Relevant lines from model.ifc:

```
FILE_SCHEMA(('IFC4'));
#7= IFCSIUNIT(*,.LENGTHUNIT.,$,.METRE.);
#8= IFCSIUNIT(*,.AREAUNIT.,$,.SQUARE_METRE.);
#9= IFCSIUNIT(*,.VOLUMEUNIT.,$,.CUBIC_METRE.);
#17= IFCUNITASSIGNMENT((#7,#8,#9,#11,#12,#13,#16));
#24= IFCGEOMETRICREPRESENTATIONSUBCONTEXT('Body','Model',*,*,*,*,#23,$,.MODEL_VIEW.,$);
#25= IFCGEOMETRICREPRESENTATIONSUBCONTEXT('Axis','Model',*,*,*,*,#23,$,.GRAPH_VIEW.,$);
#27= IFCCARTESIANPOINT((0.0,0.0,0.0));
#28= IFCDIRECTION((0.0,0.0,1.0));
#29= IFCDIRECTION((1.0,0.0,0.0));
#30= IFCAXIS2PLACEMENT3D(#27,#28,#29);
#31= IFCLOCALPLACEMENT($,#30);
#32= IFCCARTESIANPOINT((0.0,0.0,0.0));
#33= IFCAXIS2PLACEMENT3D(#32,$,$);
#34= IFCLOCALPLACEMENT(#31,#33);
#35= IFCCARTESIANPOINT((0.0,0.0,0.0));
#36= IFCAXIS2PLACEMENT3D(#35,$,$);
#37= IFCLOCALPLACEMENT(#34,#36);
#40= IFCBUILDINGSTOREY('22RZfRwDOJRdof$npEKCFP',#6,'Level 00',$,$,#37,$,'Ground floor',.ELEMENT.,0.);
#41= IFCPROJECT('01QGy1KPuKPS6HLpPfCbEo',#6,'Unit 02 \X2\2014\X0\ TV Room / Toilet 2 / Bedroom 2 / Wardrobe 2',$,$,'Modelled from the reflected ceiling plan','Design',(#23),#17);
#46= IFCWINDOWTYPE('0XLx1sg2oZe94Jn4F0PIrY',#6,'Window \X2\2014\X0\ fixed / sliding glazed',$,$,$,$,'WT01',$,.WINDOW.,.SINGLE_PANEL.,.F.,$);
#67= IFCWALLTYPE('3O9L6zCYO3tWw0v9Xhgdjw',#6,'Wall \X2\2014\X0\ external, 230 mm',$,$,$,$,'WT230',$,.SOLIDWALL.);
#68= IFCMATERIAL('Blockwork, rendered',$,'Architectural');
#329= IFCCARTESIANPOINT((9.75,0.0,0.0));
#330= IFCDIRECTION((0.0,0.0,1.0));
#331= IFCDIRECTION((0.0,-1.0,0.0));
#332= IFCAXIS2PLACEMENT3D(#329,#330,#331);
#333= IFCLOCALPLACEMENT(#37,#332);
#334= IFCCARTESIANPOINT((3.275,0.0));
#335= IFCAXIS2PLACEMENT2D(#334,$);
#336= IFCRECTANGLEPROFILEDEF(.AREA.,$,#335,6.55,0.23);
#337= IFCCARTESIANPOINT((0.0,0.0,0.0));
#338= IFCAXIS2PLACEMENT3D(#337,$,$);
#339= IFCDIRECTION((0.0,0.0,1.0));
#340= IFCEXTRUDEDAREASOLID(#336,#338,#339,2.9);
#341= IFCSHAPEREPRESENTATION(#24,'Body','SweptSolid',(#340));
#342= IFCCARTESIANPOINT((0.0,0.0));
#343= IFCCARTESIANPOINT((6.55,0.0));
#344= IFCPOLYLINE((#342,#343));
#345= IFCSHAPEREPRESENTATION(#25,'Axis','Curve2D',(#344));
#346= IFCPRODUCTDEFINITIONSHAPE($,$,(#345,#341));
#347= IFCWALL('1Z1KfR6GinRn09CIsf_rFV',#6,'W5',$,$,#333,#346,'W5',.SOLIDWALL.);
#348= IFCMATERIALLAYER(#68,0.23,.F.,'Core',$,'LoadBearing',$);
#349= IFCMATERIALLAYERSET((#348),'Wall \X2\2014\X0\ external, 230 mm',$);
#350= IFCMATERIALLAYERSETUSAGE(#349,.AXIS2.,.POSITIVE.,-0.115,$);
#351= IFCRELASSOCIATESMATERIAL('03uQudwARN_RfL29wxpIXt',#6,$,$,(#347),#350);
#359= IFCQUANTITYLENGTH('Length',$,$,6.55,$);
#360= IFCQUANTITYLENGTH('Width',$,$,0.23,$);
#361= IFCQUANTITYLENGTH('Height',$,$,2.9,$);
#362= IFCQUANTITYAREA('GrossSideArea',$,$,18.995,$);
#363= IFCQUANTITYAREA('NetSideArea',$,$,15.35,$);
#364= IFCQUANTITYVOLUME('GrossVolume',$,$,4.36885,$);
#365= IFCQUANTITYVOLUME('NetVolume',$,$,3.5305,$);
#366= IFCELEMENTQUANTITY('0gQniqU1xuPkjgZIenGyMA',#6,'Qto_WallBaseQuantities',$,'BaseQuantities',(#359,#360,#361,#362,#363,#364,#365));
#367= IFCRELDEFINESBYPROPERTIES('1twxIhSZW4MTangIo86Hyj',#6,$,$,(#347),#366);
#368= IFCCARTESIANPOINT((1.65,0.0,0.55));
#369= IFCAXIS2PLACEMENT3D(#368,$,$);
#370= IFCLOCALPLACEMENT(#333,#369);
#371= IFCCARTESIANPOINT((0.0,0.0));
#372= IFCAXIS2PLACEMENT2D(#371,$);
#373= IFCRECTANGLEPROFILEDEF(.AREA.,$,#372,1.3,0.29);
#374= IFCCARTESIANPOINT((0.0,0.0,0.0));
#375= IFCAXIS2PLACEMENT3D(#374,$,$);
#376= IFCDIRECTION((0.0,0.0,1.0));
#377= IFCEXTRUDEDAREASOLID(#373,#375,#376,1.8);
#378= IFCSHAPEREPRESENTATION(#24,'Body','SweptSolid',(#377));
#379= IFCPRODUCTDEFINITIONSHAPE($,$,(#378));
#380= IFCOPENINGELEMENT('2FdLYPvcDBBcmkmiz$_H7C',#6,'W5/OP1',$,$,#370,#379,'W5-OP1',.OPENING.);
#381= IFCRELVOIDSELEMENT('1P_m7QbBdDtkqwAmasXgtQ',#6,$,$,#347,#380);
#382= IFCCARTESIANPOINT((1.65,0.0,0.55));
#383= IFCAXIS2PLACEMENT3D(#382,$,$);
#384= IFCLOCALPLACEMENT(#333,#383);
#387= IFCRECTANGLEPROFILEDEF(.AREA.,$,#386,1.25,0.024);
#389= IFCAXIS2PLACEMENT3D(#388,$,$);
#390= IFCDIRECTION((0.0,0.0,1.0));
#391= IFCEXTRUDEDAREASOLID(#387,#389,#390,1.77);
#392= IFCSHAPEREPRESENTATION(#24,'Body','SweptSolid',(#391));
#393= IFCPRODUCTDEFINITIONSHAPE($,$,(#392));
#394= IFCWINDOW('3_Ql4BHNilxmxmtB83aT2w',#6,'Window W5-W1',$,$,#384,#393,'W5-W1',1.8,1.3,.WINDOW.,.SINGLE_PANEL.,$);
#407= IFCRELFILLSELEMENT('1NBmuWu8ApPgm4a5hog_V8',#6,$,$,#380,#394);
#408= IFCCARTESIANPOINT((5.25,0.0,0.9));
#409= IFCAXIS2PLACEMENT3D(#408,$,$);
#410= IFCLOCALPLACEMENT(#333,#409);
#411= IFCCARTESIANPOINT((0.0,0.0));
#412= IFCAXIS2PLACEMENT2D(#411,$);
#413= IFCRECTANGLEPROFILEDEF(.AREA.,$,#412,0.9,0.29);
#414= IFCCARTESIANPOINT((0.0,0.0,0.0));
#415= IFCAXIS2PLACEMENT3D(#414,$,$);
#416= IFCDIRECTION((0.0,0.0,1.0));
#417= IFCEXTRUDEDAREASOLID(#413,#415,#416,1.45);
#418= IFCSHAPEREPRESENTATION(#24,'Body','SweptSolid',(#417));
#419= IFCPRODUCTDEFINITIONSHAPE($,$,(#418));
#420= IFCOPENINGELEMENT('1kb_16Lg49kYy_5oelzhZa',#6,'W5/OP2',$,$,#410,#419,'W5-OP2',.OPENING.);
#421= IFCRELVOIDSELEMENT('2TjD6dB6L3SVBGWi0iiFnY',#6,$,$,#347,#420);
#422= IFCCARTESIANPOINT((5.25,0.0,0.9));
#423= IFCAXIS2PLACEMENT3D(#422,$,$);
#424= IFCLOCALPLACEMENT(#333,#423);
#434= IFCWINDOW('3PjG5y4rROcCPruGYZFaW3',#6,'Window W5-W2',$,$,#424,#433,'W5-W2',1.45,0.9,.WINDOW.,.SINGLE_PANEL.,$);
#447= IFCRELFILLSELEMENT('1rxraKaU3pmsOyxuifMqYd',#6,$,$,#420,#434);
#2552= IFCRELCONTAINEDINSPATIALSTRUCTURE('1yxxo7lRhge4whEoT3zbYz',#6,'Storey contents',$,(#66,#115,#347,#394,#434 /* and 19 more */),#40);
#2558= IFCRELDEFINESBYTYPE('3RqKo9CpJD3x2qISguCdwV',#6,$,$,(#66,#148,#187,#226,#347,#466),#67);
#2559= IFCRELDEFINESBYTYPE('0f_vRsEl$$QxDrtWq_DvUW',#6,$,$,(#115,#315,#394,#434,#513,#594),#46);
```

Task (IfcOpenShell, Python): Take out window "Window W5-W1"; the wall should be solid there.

```python
import ifcopenshell
import ifcopenshell.api.feature
import ifcopenshell.api.pset
import ifcopenshell.api.root
import ifcopenshell.geom
import ifcopenshell.util.element
import ifcopenshell.util.shape
import ifcopenshell.util.unit

model = ifcopenshell.open("model.ifc")
area_scale = ifcopenshell.util.unit.calculate_unit_scale(model, "AREAUNIT")
volume_scale = ifcopenshell.util.unit.calculate_unit_scale(model, "VOLUMEUNIT")
settings = ifcopenshell.geom.settings()


def volume(element):
    """Net volume in cubic metres, openings subtracted."""
    shape = ifcopenshell.geom.create_shape(settings, element)
    return ifcopenshell.util.shape.get_volume(shape.geometry)


window = model.by_guid("3_Ql4BHNilxmxmtB83aT2w")
opening = window.FillsVoids[0].RelatingOpeningElement
wall = opening.VoidsElements[0].RelatingBuildingElement
before = volume(wall)

ifcopenshell.api.root.remove_product(model, product=window)
ifcopenshell.api.feature.remove_feature(model, feature=opening)

after = volume(wall)
thickness = 0.23  # wall thickness in metres

# Update the wall's stored quantities.
qto = model.by_id(ifcopenshell.util.element.get_pset(wall, "Qto_WallBaseQuantities", should_inherit=False)["id"])
ifcopenshell.api.pset.edit_qto(model, qto=qto, properties={
    "NetSideArea": after / thickness / area_scale,
    "NetVolume": after / volume_scale,
})

print(f"wall volume {before:.3f} -> {after:.3f} m3")

model.write("model_rev.ifc")
```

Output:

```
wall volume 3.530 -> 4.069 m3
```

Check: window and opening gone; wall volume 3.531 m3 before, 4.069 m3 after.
